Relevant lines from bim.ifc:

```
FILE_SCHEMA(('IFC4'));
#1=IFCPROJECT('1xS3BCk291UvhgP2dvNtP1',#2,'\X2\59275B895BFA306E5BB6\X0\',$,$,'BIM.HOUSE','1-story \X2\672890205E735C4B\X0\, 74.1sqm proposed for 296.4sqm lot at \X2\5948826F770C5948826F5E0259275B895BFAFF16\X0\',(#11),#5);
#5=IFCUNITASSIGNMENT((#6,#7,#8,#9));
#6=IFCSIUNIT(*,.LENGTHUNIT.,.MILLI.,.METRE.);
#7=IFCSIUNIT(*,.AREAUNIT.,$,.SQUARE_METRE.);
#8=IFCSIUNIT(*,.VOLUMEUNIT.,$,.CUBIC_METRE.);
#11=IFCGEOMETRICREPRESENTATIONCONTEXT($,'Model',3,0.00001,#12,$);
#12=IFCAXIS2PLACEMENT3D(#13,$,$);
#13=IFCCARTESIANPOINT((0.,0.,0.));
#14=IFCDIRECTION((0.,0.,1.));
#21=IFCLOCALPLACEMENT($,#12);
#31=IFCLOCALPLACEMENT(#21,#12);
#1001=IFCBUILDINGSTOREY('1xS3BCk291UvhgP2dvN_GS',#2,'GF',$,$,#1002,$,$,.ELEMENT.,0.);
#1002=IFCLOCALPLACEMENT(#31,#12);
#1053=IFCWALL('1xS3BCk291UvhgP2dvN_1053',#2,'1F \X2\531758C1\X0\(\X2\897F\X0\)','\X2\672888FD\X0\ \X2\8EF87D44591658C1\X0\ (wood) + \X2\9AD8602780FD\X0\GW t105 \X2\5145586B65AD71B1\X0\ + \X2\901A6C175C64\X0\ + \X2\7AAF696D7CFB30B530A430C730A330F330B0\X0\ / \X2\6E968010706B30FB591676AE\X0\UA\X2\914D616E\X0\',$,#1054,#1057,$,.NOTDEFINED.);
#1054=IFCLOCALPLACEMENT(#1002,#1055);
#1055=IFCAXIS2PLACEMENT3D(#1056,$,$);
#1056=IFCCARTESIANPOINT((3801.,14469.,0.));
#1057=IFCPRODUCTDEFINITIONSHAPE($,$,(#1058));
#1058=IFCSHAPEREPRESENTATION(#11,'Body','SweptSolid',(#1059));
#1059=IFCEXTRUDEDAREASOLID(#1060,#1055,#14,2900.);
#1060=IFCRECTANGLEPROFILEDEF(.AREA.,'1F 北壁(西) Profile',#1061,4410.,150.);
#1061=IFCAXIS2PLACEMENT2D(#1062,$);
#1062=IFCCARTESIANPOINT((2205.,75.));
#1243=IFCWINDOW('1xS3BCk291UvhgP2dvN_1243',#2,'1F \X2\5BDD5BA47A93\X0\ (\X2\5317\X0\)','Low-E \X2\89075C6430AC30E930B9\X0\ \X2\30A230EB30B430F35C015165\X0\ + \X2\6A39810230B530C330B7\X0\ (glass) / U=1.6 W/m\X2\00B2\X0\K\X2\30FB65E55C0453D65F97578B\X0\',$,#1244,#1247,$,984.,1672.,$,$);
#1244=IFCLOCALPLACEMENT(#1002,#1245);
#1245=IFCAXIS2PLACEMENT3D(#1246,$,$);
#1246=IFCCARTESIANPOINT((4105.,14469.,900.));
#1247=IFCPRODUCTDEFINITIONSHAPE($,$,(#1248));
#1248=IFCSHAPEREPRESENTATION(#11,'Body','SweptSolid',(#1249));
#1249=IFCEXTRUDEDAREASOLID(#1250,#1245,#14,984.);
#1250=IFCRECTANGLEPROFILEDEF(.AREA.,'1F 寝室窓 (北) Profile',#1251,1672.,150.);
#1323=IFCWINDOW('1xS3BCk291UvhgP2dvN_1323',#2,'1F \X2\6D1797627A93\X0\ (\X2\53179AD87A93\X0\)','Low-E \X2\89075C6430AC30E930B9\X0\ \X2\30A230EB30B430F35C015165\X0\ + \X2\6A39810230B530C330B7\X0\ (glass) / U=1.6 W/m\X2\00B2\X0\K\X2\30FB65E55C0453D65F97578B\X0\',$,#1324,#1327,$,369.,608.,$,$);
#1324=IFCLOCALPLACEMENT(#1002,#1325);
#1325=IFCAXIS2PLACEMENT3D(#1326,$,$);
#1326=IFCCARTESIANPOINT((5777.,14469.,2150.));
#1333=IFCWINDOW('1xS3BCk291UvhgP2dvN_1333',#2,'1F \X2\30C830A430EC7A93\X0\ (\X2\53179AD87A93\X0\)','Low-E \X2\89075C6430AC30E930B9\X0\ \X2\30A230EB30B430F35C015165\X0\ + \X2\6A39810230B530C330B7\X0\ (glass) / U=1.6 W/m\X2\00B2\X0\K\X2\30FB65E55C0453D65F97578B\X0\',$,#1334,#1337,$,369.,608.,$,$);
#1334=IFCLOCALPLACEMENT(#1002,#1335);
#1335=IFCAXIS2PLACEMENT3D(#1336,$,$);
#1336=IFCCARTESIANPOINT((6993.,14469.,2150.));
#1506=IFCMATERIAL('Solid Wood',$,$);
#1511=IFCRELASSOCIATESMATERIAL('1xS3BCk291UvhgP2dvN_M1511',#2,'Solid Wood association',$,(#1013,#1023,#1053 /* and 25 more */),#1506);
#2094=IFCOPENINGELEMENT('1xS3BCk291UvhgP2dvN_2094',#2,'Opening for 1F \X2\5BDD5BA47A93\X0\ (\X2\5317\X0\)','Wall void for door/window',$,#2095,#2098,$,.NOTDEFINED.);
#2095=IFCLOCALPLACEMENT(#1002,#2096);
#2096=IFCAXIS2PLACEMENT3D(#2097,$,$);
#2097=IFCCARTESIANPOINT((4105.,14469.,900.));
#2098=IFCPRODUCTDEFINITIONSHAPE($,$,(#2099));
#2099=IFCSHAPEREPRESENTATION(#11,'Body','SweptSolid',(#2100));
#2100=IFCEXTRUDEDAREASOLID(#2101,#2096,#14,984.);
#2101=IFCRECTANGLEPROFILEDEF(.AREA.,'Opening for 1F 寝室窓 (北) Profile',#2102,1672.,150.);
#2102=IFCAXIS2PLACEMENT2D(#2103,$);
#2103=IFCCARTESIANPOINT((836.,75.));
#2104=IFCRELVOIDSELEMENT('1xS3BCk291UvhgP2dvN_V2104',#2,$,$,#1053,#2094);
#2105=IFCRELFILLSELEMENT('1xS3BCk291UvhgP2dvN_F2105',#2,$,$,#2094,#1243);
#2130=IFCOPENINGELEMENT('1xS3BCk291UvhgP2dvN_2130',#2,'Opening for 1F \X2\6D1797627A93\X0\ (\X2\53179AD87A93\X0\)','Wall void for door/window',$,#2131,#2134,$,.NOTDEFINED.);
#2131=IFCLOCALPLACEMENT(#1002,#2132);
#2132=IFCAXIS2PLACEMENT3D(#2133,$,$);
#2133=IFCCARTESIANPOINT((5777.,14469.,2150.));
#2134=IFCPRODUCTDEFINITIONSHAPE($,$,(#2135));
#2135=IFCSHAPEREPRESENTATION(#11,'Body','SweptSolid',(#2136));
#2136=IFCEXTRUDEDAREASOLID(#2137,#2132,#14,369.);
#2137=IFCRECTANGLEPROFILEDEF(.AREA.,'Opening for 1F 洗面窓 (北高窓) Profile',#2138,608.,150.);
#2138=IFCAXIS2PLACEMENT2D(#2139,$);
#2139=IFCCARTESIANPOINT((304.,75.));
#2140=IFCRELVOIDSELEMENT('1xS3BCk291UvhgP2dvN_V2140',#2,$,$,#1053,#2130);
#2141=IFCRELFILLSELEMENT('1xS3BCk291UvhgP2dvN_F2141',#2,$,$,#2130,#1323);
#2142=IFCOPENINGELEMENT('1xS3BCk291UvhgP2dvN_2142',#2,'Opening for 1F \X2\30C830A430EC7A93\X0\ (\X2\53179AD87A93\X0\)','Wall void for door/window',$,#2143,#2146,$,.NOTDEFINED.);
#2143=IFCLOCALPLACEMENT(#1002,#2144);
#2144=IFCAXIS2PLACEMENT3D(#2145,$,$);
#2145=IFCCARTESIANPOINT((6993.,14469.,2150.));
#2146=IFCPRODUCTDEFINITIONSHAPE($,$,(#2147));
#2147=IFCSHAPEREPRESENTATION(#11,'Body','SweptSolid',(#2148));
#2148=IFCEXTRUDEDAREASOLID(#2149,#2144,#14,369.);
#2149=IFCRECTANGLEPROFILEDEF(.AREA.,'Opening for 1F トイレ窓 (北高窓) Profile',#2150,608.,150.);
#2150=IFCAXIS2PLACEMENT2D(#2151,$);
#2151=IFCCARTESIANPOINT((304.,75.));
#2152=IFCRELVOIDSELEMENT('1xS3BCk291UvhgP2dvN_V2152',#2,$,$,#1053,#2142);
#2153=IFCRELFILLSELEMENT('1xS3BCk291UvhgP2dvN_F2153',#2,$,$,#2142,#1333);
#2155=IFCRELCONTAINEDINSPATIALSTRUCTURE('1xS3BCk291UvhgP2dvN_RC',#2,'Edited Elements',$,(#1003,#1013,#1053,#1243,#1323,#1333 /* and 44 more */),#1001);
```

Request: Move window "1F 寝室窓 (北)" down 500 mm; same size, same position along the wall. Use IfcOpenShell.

```python
import numpy as np
import ifcopenshell
import ifcopenshell.api.geometry
import ifcopenshell.util.placement
import ifcopenshell.util.unit

model = ifcopenshell.open("bim.ifc")
unit_scale = ifcopenshell.util.unit.calculate_unit_scale(model)

window = model.by_guid("1xS3BCk291UvhgP2dvN_1243")
opening = window.FillsVoids[0].RelatingOpeningElement
dz = -0.5 / unit_scale

shift = np.array([0.0, 0.0, dz])
# The window is not placed relative to its opening, so move both.
for product in (opening, window):
    matrix = ifcopenshell.util.placement.get_local_placement(product.ObjectPlacement)
    matrix[:3, 3] += shift
    ifcopenshell.api.geometry.edit_object_placement(model, product=product, matrix=matrix, is_si=False)

print(f"moved by {dz * unit_scale:+.3f} m")

model.write("bim-out.ifc")
```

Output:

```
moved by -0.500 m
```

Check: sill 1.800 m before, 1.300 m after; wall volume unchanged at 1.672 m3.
